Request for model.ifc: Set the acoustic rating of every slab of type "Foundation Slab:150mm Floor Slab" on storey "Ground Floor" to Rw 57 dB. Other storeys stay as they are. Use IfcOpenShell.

First a look at what the model holds.

```python
import ifcopenshell
import ifcopenshell.util.element

model = ifcopenshell.open("model.ifc")
print(model.schema)
storey = next(s for s in model.by_type("IfcBuildingStorey") if s.Name == "Ground Floor")
slabs = [e for e in ifcopenshell.util.element.get_decomposition(storey) if e.is_a("IfcSlab")]
seen = {}
for e in slabs:
    element_type = ifcopenshell.util.element.get_type(e)
    key = (element_type.Name if element_type != e and element_type else None, ifcopenshell.util.element.get_pset(e, "Pset_SlabCommon", "AcousticRating"))
    seen[key] = seen.get(key, 0) + 1
for (name, value), count in sorted(seen.items(), key=str):
    print(count, "x", name, "|", value)
```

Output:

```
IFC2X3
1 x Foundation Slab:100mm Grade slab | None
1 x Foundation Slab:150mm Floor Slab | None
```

```python
import ifcopenshell
import ifcopenshell.api.pset
import ifcopenshell.util.element

model = ifcopenshell.open("model.ifc")

storey = next(s for s in model.by_type("IfcBuildingStorey") if s.Name == "Ground Floor")
slabs = [e for e in ifcopenshell.util.element.get_decomposition(storey) if e.is_a("IfcSlab")]

count = 0
for e in slabs:
    element_type = ifcopenshell.util.element.get_type(e)
    if element_type in (None, e) or element_type.Name != "Foundation Slab:150mm Floor Slab":
        continue
    # add_pset returns the element's existing set when there is one.
    pset = ifcopenshell.api.pset.add_pset(model, product=e, name="Pset_SlabCommon")
    ifcopenshell.api.pset.edit_pset(model, pset=pset, properties={"AcousticRating": "Rw 57 dB"})
    count += 1

print(count, "slabs updated")

model.write("model-out.ifc")
```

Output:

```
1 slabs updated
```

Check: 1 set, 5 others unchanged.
